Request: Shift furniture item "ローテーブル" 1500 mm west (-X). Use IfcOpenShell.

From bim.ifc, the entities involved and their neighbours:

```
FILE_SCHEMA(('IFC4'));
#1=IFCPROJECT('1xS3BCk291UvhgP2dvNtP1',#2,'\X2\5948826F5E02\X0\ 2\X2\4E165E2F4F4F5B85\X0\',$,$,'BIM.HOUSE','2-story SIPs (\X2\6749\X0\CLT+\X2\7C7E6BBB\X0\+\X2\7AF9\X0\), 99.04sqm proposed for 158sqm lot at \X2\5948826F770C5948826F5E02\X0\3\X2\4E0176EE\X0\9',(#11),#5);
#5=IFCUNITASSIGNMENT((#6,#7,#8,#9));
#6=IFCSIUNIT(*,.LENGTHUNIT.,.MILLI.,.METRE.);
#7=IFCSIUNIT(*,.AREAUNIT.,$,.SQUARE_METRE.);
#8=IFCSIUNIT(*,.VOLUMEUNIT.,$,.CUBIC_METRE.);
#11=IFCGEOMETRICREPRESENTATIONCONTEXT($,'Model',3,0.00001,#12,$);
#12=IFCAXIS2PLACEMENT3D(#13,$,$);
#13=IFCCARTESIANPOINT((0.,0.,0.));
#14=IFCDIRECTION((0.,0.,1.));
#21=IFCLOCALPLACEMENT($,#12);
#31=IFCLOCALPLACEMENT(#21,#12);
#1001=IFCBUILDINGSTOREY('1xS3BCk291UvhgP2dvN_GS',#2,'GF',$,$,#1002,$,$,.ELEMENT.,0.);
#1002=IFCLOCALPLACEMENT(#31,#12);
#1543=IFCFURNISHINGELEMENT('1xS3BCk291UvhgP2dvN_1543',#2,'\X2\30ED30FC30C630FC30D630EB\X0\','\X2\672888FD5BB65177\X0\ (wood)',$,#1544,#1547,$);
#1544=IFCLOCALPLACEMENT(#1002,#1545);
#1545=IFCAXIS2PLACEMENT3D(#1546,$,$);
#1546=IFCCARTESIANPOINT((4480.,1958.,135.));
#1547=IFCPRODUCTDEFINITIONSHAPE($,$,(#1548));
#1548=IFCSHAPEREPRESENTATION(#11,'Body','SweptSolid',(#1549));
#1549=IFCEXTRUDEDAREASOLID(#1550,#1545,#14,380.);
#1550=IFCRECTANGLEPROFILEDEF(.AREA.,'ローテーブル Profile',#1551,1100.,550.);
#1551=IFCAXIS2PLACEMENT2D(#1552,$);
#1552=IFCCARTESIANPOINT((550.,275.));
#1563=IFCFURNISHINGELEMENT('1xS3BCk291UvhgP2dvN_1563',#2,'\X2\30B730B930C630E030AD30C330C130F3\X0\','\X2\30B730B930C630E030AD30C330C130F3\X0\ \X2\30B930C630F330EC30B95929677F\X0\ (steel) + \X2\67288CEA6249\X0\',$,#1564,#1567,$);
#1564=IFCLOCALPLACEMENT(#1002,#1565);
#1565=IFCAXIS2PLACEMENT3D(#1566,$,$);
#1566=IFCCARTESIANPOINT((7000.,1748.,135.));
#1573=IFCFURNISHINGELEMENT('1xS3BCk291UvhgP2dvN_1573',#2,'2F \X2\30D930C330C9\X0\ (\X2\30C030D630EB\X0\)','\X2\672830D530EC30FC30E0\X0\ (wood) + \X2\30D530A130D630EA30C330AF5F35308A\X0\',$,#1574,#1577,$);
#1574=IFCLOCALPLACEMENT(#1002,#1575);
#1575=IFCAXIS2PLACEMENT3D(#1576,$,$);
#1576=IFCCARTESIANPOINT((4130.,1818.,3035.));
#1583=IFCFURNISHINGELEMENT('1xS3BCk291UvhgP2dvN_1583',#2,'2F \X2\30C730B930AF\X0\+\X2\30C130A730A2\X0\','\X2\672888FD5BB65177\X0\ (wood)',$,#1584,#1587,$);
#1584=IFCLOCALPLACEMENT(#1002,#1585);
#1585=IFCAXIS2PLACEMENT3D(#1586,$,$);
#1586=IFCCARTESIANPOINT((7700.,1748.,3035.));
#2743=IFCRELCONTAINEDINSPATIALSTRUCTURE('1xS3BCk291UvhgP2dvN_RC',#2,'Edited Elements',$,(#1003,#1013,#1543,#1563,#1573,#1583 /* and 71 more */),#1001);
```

```python
import ifcopenshell
import ifcopenshell.api.geometry
import ifcopenshell.util.placement
import ifcopenshell.util.unit

model = ifcopenshell.open("bim.ifc")
unit_scale = ifcopenshell.util.unit.calculate_unit_scale(model)

item = model.by_id(1543)
matrix = ifcopenshell.util.placement.get_local_placement(item.ObjectPlacement)
matrix[0, 3] -= 1.5 / unit_scale
ifcopenshell.api.geometry.edit_object_placement(model, product=item, matrix=matrix, is_si=False)

print(ifcopenshell.util.placement.get_local_placement(item.ObjectPlacement).round(3) + 0.0)

model.write("bim-out.ifc")
```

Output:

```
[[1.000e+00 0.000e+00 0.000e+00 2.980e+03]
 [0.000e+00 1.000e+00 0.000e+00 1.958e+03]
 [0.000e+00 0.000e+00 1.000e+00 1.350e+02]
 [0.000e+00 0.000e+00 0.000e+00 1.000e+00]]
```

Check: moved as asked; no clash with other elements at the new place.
